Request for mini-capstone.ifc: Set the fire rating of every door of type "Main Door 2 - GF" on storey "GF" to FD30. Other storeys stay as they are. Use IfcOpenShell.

First a look at what the model holds.

```python
import ifcopenshell
import ifcopenshell.util.element

model = ifcopenshell.open("mini-capstone.ifc")
print(model.schema)
storey = next(s for s in model.by_type("IfcBuildingStorey") if s.Name == "GF")
doors = [e for e in ifcopenshell.util.element.get_decomposition(storey) if e.is_a("IfcDoor")]
seen = {}
for e in doors:
    element_type = ifcopenshell.util.element.get_type(e)
    key = (element_type.Name if element_type != e and element_type else None, ifcopenshell.util.element.get_pset(e, "Pset_DoorCommon", "FireRating"))
    seen[key] = seen.get(key, 0) + 1
for (name, value), count in sorted(seen.items(), key=str):
    print(count, "x", name, "|", value)
```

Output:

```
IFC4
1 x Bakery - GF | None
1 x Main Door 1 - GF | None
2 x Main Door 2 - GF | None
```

```python
import ifcopenshell
import ifcopenshell.api.pset
import ifcopenshell.util.element

model = ifcopenshell.open("mini-capstone.ifc")

storey = next(s for s in model.by_type("IfcBuildingStorey") if s.Name == "GF")
doors = [e for e in ifcopenshell.util.element.get_decomposition(storey) if e.is_a("IfcDoor")]

count = 0
for e in doors:
    element_type = ifcopenshell.util.element.get_type(e)
    if element_type in (None, e) or element_type.Name != "Main Door 2 - GF":
        continue
    # add_pset returns the element's existing set when there is one.
    pset = ifcopenshell.api.pset.add_pset(model, product=e, name="Pset_DoorCommon")
    ifcopenshell.api.pset.edit_pset(model, pset=pset, properties={"FireRating": "FD30"})
    count += 1

print(count, "doors updated")

model.write("mini-capstone_edited.ifc")
```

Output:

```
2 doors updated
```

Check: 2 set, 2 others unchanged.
